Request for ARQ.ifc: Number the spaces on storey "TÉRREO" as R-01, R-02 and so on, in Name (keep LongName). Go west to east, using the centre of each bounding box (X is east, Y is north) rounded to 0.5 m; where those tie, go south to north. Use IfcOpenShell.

First a look at what the model holds.

```python
import ifcopenshell
import ifcopenshell.util.element
import ifcopenshell.util.placement

model = ifcopenshell.open("ARQ.ifc")
print(model.schema)
storey = next(s for s in model.by_type("IfcBuildingStorey") if s.Name == "TÉRREO")
spaces = [e for e in ifcopenshell.util.element.get_decomposition(storey) if e.is_a("IfcSpace")]
for e in sorted(spaces, key=lambda e: e.id()):
    origin = ifcopenshell.util.placement.get_local_placement(e.ObjectPlacement)[:3, 3]
    print(e.id(), e.Name, e.LongName, origin.round(2) + 0.0, sep=" | ")
```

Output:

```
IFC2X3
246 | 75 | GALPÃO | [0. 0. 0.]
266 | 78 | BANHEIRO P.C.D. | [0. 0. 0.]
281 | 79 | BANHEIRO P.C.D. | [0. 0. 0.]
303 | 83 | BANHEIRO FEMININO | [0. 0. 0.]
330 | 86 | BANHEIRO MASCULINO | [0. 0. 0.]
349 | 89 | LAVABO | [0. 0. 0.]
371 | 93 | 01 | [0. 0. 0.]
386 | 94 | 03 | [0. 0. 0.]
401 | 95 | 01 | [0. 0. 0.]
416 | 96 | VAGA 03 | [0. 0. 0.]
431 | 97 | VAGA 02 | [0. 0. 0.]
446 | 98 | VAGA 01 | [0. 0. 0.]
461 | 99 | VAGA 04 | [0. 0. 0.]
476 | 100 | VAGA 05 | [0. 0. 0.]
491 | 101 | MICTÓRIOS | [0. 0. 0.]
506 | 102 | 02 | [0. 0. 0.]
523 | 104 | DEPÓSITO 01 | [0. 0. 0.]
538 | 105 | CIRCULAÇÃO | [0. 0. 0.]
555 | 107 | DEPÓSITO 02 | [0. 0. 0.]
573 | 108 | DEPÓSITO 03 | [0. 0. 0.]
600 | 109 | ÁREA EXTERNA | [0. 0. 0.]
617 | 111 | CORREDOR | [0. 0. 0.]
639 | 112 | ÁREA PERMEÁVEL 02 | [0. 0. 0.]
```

```python
import ifcopenshell
import ifcopenshell.geom
import ifcopenshell.util.element
import ifcopenshell.util.shape

model = ifcopenshell.open("ARQ.ifc")
settings = ifcopenshell.geom.settings()
settings.set("use-world-coords", True)


def centre(element):
    shape = ifcopenshell.geom.create_shape(settings, element)
    return ifcopenshell.util.shape.get_bbox_centroid(shape.geometry)


storey = next(s for s in model.by_type("IfcBuildingStorey") if s.Name == "TÉRREO")
spaces = [e for e in ifcopenshell.util.element.get_decomposition(storey) if e.is_a("IfcSpace")]

# Insertion points can sit at a corner or the storey origin, so sort by the geometry (in metres).
centres = {e: centre(e) for e in spaces}
spaces.sort(key=lambda e: (round(centres[e][0] / 0.5), centres[e][1]))

for i, e in enumerate(spaces, start=1):
    number = f"R-{i:02d}"
    e.Name = number
    print(e.id(), number)

model.write("ARQ-out.ifc")
```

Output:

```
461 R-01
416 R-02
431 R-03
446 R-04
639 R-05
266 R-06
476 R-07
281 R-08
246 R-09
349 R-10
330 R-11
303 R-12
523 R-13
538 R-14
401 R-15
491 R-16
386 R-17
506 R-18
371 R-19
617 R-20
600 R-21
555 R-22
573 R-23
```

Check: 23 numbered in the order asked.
